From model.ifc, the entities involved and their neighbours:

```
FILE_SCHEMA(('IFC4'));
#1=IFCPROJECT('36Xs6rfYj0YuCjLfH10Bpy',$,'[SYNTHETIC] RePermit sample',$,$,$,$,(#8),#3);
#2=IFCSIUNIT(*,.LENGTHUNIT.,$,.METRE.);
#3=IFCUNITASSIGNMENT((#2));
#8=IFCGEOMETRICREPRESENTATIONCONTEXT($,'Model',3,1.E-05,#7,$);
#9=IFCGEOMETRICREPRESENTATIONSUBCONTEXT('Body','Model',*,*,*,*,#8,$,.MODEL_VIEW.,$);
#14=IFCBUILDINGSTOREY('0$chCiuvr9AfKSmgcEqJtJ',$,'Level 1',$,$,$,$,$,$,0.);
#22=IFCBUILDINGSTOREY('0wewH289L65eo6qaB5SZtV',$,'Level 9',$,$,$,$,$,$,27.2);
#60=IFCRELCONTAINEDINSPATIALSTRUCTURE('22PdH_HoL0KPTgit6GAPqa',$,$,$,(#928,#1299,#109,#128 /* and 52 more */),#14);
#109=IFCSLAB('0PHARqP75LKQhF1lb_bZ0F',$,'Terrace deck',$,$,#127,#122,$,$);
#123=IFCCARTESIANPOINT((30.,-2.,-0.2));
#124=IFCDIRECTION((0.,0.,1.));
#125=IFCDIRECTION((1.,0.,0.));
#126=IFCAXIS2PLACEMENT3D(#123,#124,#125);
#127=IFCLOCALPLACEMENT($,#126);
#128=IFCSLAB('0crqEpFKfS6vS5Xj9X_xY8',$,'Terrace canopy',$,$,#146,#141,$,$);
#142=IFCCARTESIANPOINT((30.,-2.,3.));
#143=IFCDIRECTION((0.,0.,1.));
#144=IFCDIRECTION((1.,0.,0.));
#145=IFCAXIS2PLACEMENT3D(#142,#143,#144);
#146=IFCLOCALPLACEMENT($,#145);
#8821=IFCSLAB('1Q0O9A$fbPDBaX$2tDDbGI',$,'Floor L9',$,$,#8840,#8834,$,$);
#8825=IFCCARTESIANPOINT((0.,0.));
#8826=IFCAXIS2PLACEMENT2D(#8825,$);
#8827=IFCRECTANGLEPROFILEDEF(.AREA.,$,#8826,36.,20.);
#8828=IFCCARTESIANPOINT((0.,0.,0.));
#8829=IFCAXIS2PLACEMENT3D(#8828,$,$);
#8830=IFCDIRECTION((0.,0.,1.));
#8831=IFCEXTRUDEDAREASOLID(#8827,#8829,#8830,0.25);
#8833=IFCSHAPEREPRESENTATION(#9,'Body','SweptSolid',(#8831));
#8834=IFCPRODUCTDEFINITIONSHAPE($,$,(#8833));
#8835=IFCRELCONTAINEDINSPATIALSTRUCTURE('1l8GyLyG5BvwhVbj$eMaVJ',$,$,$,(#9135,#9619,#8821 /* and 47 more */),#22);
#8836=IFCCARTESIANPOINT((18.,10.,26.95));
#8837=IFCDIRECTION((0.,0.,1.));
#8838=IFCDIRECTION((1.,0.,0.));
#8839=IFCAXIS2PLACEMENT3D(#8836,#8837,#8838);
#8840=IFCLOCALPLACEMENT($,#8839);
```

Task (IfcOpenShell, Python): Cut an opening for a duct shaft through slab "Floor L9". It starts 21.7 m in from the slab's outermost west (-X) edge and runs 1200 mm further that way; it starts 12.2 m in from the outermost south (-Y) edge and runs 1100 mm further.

```python
import numpy as np
import ifcopenshell
import ifcopenshell.api.feature
import ifcopenshell.api.geometry
import ifcopenshell.api.root
import ifcopenshell.geom
import ifcopenshell.util.placement
import ifcopenshell.util.representation
import ifcopenshell.util.shape
import ifcopenshell.util.unit

model = ifcopenshell.open("model.ifc")
unit_scale = ifcopenshell.util.unit.calculate_unit_scale(model)
settings = ifcopenshell.geom.settings()


def volume(element):
    """Net volume in cubic metres, openings subtracted."""
    shape = ifcopenshell.geom.create_shape(settings, element)
    return ifcopenshell.util.shape.get_volume(shape.geometry)


slab = model.by_id(8821)
before = volume(slab)

# Extent in the slab's own axes, in metres. The edges named are its -X and -Y sides.
slab_shape = ifcopenshell.geom.create_shape(settings, slab)
vertices = ifcopenshell.util.shape.get_vertices(slab_shape.geometry)
x_min, y_min, bottom = vertices.min(axis=0)
top = vertices[:, 2].max()

opening = ifcopenshell.api.root.create_entity(model, ifc_class="IfcOpeningElement", name="Duct shaft opening", predefined_type="OPENING")
context = ifcopenshell.util.representation.get_context(model, "Model", "Body", "MODEL_VIEW")
width, depth = 1.2, 1.1
outline = [(0.0, 0.0), (width, 0.0), (width, depth), (0.0, depth), (0.0, 0.0)]
# Overshoot both faces by 50 mm so the cut is clean.
shape = ifcopenshell.api.geometry.add_slab_representation(
    model, context=context, depth=top - bottom + 0.1, polyline=outline
)
ifcopenshell.api.geometry.assign_representation(model, product=opening, representation=shape)

matrix = ifcopenshell.util.placement.get_local_placement(slab.ObjectPlacement)
matrix[:, 3] = matrix @ np.append(np.array([x_min + 21.7, y_min + 12.2, bottom - 0.05]) / unit_scale, 1.0)
ifcopenshell.api.geometry.edit_object_placement(model, product=opening, matrix=matrix, is_si=False)
ifcopenshell.api.feature.add_feature(model, feature=opening, element=slab)

after = volume(slab)

print(f"slab volume {before:.3f} -> {after:.3f} m3")

model.write("model_v2.ifc")
```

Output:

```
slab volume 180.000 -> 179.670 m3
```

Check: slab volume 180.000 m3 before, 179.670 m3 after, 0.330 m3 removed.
